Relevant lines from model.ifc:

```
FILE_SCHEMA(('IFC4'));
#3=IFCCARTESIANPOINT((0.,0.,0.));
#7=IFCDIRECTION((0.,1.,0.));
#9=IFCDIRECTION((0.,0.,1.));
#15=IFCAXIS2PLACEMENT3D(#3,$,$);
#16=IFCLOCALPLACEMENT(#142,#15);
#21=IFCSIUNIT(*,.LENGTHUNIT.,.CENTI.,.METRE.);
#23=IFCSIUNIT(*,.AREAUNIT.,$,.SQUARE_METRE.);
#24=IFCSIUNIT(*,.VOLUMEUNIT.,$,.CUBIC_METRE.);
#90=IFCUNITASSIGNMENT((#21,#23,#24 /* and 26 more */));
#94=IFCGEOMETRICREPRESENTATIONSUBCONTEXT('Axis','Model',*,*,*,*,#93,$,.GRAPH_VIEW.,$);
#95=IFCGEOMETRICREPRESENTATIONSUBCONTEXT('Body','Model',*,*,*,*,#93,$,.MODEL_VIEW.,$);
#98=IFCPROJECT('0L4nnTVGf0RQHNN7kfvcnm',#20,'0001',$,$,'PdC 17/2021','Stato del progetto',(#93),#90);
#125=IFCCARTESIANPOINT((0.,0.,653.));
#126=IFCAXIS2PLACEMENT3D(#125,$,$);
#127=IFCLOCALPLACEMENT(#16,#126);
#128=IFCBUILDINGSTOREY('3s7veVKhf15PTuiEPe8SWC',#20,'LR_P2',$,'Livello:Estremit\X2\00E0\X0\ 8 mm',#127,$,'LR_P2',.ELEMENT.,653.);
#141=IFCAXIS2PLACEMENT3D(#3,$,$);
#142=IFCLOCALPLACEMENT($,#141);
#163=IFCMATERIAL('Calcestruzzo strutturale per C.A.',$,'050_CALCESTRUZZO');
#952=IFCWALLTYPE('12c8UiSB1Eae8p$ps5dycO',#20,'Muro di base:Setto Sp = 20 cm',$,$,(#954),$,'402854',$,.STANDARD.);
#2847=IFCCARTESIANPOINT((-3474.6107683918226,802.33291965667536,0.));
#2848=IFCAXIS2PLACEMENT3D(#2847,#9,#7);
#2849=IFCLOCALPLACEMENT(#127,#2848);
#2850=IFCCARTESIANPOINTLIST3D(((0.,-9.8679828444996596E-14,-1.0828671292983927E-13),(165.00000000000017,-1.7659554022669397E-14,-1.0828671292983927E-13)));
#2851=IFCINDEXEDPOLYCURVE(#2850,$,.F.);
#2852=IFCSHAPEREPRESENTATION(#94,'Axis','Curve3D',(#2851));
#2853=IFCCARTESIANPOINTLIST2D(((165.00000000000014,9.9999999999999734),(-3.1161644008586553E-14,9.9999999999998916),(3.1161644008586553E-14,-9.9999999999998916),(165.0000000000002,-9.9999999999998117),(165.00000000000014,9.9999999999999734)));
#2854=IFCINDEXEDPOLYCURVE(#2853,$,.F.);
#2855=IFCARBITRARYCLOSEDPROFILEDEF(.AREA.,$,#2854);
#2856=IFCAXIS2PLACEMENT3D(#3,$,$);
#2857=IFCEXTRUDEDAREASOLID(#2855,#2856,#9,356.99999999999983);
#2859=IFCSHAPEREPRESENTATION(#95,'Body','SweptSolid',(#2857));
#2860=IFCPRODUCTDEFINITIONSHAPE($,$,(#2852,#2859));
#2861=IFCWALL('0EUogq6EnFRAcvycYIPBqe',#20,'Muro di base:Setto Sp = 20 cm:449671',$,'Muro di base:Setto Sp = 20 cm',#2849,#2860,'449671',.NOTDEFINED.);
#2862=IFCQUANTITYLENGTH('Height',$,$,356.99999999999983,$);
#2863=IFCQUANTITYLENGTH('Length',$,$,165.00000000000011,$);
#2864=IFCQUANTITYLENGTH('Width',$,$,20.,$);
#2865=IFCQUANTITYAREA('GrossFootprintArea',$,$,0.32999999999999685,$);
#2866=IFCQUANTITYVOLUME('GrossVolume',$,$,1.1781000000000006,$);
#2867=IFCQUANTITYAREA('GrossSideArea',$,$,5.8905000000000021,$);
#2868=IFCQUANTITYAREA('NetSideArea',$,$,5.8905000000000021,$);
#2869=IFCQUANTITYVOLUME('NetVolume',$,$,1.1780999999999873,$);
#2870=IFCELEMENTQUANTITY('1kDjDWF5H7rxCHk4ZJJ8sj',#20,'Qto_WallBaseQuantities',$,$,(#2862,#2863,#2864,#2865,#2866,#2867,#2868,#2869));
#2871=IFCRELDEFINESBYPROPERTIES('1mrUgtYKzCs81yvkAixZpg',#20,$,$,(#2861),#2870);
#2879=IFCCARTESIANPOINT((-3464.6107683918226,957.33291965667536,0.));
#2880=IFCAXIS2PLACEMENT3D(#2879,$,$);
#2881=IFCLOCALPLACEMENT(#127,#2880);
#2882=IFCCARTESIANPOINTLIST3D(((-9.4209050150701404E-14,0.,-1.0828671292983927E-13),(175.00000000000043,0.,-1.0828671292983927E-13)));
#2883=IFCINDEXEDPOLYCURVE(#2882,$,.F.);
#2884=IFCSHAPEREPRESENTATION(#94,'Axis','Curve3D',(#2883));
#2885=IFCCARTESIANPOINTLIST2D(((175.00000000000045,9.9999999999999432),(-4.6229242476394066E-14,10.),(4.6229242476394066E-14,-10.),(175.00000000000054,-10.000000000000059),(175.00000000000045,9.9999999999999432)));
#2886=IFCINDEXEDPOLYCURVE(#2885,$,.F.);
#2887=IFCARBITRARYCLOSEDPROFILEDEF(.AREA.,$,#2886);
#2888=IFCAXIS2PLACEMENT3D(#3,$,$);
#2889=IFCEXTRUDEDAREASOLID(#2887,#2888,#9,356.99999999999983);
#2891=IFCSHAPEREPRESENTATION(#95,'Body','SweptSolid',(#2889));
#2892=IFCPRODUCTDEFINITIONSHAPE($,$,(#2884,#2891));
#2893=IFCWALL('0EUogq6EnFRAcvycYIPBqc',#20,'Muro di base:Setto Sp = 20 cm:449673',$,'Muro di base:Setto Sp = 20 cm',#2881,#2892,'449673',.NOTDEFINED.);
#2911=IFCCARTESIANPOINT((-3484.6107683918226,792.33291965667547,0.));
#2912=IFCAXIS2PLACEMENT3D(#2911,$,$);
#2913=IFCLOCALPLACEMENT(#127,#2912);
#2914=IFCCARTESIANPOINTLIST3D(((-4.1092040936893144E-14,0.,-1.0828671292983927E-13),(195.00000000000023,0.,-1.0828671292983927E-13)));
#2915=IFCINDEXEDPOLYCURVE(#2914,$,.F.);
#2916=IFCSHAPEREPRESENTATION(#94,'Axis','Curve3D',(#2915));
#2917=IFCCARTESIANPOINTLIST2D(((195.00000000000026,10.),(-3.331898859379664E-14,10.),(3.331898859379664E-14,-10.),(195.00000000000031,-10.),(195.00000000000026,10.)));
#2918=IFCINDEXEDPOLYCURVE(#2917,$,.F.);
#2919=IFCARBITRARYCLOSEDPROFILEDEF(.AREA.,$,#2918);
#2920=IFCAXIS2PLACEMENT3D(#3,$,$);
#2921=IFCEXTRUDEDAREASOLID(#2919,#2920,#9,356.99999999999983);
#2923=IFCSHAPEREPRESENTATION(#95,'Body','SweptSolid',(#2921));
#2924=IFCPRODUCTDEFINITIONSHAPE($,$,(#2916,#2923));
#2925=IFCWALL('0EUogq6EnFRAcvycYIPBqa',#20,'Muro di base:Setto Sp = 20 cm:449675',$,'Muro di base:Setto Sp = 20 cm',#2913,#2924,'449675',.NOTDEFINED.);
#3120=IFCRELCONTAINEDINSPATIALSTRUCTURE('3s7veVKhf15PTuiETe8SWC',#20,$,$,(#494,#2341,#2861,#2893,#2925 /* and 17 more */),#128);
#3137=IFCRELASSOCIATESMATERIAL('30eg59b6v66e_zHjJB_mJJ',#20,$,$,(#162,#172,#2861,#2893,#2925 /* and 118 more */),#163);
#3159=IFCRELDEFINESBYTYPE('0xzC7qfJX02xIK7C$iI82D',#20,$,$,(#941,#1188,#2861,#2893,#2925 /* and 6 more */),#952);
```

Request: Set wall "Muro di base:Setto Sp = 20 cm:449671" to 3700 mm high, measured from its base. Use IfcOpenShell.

```python
import ifcopenshell
import ifcopenshell.api.pset
import ifcopenshell.geom
import ifcopenshell.util.element
import ifcopenshell.util.representation
import ifcopenshell.util.shape
import ifcopenshell.util.unit

model = ifcopenshell.open("model.ifc")
unit_scale = ifcopenshell.util.unit.calculate_unit_scale(model)
area_scale = ifcopenshell.util.unit.calculate_unit_scale(model, "AREAUNIT")
volume_scale = ifcopenshell.util.unit.calculate_unit_scale(model, "VOLUMEUNIT")
settings = ifcopenshell.geom.settings()


def volume(element):
    """Net volume in cubic metres, openings subtracted."""
    shape = ifcopenshell.geom.create_shape(settings, element)
    return ifcopenshell.util.shape.get_volume(shape.geometry)


wall = model.by_id(2861)
before = volume(wall)

body = ifcopenshell.util.representation.get_representation(wall, "Model", "Body")
solid = body.Items[0]
old_height = solid.Depth
solid.Depth = 3.7 / unit_scale
after = volume(wall)
thickness = 0.2  # wall thickness in metres

# Update the stored height, areas and volumes.
qto = model.by_id(ifcopenshell.util.element.get_pset(wall, "Qto_WallBaseQuantities", should_inherit=False)["id"])
ifcopenshell.api.pset.edit_qto(model, qto=qto, properties={
    "Height": solid.Depth,
    "GrossVolume": ifcopenshell.util.element.get_pset(wall, "Qto_WallBaseQuantities", "GrossVolume") * solid.Depth / old_height,
    "GrossSideArea": ifcopenshell.util.element.get_pset(wall, "Qto_WallBaseQuantities", "GrossSideArea") * solid.Depth / old_height,
    "NetSideArea": after / thickness / area_scale,
    "NetVolume": after / volume_scale,
})

print(f"height {old_height:g} -> {solid.Depth:g}, volume {before:.3f} -> {after:.3f} m3")

model.write("model_updated.ifc")
```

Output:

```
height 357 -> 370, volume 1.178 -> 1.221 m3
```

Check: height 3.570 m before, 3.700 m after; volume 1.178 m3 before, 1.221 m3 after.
